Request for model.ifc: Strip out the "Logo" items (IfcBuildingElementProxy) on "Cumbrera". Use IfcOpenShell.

First a look at what the model holds.

```python
import ifcopenshell
import ifcopenshell.util.element

model = ifcopenshell.open("model.ifc")
print(model.schema)
storey = next(s for s in model.by_type("IfcBuildingStorey") if s.Name == "Cumbrera")
proxies = [e for e in ifcopenshell.util.element.get_decomposition(storey) if e.is_a("IfcBuildingElementProxy")]
seen = {}
for e in proxies:
    element_type = ifcopenshell.util.element.get_type(e)
    name = element_type.Name if element_type not in (None, e) else None
    seen[name] = seen.get(name, 0) + 1
for name, count in sorted(seen.items(), key=str):
    print(count, "x", name)
```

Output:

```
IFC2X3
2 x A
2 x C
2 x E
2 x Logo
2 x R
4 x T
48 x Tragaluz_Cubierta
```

```python
import ifcopenshell
import ifcopenshell.api.root
import ifcopenshell.util.element

model = ifcopenshell.open("model.ifc")

storey = next(s for s in model.by_type("IfcBuildingStorey") if s.Name == "Cumbrera")
proxies = [e for e in ifcopenshell.util.element.get_decomposition(storey) if e.is_a("IfcBuildingElementProxy")]
targets = [e for e in proxies if (t := ifcopenshell.util.element.get_type(e)) not in (None, e) and t.Name == "Logo"]

for e in targets:
    ifcopenshell.api.root.remove_product(model, product=e)
print(len(targets), "removed")

model.write("model-out.ifc")
```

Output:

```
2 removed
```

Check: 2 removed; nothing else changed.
